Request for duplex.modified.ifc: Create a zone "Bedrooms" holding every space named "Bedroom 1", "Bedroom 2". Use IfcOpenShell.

First a look at what the model holds.

```python
import ifcopenshell

model = ifcopenshell.open("duplex.modified.ifc")
print(model.schema)
seen = {}
for space in model.by_type("IfcSpace"):
    seen[space.LongName] = seen.get(space.LongName, 0) + 1
for name, count in sorted(seen.items(), key=str):
    print(count, "x", name)
print("zones:", [z.Name for z in model.by_type("IfcZone")][:20])
```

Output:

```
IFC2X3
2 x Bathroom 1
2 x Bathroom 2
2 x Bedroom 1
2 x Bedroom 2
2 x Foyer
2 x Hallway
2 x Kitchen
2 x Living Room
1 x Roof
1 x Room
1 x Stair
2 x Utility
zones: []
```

```python
import ifcopenshell
import ifcopenshell.api.group
import ifcopenshell.api.root

model = ifcopenshell.open("duplex.modified.ifc")

names = {"Bedroom 1", "Bedroom 2"}
spaces = [s for s in model.by_type("IfcSpace") if s.LongName in names]

zone = ifcopenshell.api.root.create_entity(model, ifc_class="IfcZone", name="Bedrooms")
ifcopenshell.api.group.assign_group(model, products=spaces, group=zone)
print(len(spaces), "spaces in", zone.Name)

model.write("duplex.modified_v2.ifc")
```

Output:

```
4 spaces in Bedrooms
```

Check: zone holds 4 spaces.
